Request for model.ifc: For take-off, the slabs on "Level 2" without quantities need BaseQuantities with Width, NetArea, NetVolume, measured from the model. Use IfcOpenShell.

First a look at what the model holds.

```python
import ifcopenshell
import ifcopenshell.util.element
import ifcopenshell.util.unit

model = ifcopenshell.open("model.ifc")
print(model.schema)
for unit_type in ("LENGTHUNIT", "AREAUNIT", "VOLUMEUNIT"):
    print(unit_type, ifcopenshell.util.unit.calculate_unit_scale(model, unit_type))
storey = next(s for s in model.by_type("IfcBuildingStorey") if s.Name == "Level 2")
slabs = [e for e in ifcopenshell.util.element.get_decomposition(storey) if e.is_a("IfcSlab")]
for e in sorted(slabs, key=lambda e: e.id()):
    print(e.id(), e.is_a(), e.Name, list(ifcopenshell.util.element.get_psets(e, qtos_only=True)), sep=" | ")
```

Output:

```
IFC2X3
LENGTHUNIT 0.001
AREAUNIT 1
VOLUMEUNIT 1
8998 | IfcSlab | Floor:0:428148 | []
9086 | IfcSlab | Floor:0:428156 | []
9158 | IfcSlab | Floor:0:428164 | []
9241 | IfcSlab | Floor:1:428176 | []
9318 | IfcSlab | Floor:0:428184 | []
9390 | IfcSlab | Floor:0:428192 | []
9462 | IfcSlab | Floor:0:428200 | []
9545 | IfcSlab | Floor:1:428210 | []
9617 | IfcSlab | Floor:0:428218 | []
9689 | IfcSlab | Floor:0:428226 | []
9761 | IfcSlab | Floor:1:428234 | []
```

```python
import ifcopenshell
import ifcopenshell.api.pset
import ifcopenshell.geom
import ifcopenshell.util.element
import ifcopenshell.util.shape
import ifcopenshell.util.unit

model = ifcopenshell.open("model.ifc")
unit_scale = ifcopenshell.util.unit.calculate_unit_scale(model)
area_scale = ifcopenshell.util.unit.calculate_unit_scale(model, "AREAUNIT")
volume_scale = ifcopenshell.util.unit.calculate_unit_scale(model, "VOLUMEUNIT")
settings = ifcopenshell.geom.settings()

storey = next(s for s in model.by_type("IfcBuildingStorey") if s.Name == "Level 2")
slabs = [e for e in ifcopenshell.util.element.get_decomposition(storey) if e.is_a("IfcSlab")]

for e in sorted(slabs, key=lambda e: e.id()):
    if ifcopenshell.util.element.get_psets(e, qtos_only=True, should_inherit=False):
        continue
    # Geometry comes back in metres, in the element's own axes.
    shape = ifcopenshell.geom.create_shape(settings, e)
    values = {
        "Width": ifcopenshell.util.shape.get_z(shape.geometry) / unit_scale,
        "NetArea": ifcopenshell.util.shape.get_footprint_area(shape.geometry) / area_scale,
        "NetVolume": ifcopenshell.util.shape.get_volume(shape.geometry) / volume_scale,
    }
    qto = ifcopenshell.api.pset.add_qto(model, product=e, name="BaseQuantities")
    ifcopenshell.api.pset.edit_qto(model, qto=qto, properties=values)
    print(e.id(), {k: round(v, 3) for k, v in values.items()})

model.write("model_v2.ifc")
```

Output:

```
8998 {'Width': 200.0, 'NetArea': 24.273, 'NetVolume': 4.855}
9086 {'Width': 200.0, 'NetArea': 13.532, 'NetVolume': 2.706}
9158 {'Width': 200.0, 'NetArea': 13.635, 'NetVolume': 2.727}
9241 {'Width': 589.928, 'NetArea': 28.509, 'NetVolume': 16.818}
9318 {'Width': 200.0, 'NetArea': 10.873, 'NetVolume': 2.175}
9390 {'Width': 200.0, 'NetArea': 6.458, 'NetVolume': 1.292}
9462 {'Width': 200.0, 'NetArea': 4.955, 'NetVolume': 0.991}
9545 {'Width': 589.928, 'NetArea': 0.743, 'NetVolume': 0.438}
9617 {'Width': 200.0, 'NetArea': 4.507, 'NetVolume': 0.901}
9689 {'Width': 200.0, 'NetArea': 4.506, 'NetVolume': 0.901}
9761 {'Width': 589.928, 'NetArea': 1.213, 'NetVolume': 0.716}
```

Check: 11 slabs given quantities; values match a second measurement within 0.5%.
